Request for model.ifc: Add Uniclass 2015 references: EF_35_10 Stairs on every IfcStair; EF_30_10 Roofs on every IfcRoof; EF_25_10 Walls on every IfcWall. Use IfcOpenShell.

First a look at what the model holds.

```python
import ifcopenshell

model = ifcopenshell.open("model.ifc")
print(model.schema)
print("classifications:", [c.Name for c in model.by_type("IfcClassification")])
for ifc_class in ("IfcDoor", "IfcRoof", "IfcStair", "IfcWall", "IfcWindow"):
    print(ifc_class, len(model.by_type(ifc_class)))
```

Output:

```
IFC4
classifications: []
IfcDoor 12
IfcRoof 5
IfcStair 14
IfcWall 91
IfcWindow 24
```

```python
import ifcopenshell
import ifcopenshell.api.classification

model = ifcopenshell.open("model.ifc")

system = ifcopenshell.api.classification.add_classification(model, classification="Uniclass 2015")

codes = {
    "IfcStair": ("EF_35_10", "Stairs"),
    "IfcRoof": ("EF_30_10", "Roofs"),
    "IfcWall": ("EF_25_10", "Walls"),
}
for ifc_class, (code, name) in codes.items():
    products = model.by_type(ifc_class)
    ifcopenshell.api.classification.add_reference(
        model, products=products, classification=system, identification=code, name=name
    )
    print(code, len(products))

model.write("model_updated.ifc")
```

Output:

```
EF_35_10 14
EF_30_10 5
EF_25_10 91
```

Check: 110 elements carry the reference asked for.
